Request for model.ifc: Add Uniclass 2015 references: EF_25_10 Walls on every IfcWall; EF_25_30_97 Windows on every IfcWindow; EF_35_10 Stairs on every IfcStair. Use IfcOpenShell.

First a look at what the model holds.

```python
import ifcopenshell

model = ifcopenshell.open("model.ifc")
print(model.schema)
print("classifications:", [c.Name for c in model.by_type("IfcClassification")])
for ifc_class in ("IfcDoor", "IfcRoof", "IfcStair", "IfcWall", "IfcWindow"):
    print(ifc_class, len(model.by_type(ifc_class)))
```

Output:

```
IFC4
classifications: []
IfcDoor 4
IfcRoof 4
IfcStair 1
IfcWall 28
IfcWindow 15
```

```python
import ifcopenshell
import ifcopenshell.api.classification

model = ifcopenshell.open("model.ifc")

system = ifcopenshell.api.classification.add_classification(model, classification="Uniclass 2015")

codes = {
    "IfcWall": ("EF_25_10", "Walls"),
    "IfcWindow": ("EF_25_30_97", "Windows"),
    "IfcStair": ("EF_35_10", "Stairs"),
}
for ifc_class, (code, name) in codes.items():
    products = model.by_type(ifc_class)
    ifcopenshell.api.classification.add_reference(
        model, products=products, classification=system, identification=code, name=name
    )
    print(code, len(products))

model.write("model_rev.ifc")
```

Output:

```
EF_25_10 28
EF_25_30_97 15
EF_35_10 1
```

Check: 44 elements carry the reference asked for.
